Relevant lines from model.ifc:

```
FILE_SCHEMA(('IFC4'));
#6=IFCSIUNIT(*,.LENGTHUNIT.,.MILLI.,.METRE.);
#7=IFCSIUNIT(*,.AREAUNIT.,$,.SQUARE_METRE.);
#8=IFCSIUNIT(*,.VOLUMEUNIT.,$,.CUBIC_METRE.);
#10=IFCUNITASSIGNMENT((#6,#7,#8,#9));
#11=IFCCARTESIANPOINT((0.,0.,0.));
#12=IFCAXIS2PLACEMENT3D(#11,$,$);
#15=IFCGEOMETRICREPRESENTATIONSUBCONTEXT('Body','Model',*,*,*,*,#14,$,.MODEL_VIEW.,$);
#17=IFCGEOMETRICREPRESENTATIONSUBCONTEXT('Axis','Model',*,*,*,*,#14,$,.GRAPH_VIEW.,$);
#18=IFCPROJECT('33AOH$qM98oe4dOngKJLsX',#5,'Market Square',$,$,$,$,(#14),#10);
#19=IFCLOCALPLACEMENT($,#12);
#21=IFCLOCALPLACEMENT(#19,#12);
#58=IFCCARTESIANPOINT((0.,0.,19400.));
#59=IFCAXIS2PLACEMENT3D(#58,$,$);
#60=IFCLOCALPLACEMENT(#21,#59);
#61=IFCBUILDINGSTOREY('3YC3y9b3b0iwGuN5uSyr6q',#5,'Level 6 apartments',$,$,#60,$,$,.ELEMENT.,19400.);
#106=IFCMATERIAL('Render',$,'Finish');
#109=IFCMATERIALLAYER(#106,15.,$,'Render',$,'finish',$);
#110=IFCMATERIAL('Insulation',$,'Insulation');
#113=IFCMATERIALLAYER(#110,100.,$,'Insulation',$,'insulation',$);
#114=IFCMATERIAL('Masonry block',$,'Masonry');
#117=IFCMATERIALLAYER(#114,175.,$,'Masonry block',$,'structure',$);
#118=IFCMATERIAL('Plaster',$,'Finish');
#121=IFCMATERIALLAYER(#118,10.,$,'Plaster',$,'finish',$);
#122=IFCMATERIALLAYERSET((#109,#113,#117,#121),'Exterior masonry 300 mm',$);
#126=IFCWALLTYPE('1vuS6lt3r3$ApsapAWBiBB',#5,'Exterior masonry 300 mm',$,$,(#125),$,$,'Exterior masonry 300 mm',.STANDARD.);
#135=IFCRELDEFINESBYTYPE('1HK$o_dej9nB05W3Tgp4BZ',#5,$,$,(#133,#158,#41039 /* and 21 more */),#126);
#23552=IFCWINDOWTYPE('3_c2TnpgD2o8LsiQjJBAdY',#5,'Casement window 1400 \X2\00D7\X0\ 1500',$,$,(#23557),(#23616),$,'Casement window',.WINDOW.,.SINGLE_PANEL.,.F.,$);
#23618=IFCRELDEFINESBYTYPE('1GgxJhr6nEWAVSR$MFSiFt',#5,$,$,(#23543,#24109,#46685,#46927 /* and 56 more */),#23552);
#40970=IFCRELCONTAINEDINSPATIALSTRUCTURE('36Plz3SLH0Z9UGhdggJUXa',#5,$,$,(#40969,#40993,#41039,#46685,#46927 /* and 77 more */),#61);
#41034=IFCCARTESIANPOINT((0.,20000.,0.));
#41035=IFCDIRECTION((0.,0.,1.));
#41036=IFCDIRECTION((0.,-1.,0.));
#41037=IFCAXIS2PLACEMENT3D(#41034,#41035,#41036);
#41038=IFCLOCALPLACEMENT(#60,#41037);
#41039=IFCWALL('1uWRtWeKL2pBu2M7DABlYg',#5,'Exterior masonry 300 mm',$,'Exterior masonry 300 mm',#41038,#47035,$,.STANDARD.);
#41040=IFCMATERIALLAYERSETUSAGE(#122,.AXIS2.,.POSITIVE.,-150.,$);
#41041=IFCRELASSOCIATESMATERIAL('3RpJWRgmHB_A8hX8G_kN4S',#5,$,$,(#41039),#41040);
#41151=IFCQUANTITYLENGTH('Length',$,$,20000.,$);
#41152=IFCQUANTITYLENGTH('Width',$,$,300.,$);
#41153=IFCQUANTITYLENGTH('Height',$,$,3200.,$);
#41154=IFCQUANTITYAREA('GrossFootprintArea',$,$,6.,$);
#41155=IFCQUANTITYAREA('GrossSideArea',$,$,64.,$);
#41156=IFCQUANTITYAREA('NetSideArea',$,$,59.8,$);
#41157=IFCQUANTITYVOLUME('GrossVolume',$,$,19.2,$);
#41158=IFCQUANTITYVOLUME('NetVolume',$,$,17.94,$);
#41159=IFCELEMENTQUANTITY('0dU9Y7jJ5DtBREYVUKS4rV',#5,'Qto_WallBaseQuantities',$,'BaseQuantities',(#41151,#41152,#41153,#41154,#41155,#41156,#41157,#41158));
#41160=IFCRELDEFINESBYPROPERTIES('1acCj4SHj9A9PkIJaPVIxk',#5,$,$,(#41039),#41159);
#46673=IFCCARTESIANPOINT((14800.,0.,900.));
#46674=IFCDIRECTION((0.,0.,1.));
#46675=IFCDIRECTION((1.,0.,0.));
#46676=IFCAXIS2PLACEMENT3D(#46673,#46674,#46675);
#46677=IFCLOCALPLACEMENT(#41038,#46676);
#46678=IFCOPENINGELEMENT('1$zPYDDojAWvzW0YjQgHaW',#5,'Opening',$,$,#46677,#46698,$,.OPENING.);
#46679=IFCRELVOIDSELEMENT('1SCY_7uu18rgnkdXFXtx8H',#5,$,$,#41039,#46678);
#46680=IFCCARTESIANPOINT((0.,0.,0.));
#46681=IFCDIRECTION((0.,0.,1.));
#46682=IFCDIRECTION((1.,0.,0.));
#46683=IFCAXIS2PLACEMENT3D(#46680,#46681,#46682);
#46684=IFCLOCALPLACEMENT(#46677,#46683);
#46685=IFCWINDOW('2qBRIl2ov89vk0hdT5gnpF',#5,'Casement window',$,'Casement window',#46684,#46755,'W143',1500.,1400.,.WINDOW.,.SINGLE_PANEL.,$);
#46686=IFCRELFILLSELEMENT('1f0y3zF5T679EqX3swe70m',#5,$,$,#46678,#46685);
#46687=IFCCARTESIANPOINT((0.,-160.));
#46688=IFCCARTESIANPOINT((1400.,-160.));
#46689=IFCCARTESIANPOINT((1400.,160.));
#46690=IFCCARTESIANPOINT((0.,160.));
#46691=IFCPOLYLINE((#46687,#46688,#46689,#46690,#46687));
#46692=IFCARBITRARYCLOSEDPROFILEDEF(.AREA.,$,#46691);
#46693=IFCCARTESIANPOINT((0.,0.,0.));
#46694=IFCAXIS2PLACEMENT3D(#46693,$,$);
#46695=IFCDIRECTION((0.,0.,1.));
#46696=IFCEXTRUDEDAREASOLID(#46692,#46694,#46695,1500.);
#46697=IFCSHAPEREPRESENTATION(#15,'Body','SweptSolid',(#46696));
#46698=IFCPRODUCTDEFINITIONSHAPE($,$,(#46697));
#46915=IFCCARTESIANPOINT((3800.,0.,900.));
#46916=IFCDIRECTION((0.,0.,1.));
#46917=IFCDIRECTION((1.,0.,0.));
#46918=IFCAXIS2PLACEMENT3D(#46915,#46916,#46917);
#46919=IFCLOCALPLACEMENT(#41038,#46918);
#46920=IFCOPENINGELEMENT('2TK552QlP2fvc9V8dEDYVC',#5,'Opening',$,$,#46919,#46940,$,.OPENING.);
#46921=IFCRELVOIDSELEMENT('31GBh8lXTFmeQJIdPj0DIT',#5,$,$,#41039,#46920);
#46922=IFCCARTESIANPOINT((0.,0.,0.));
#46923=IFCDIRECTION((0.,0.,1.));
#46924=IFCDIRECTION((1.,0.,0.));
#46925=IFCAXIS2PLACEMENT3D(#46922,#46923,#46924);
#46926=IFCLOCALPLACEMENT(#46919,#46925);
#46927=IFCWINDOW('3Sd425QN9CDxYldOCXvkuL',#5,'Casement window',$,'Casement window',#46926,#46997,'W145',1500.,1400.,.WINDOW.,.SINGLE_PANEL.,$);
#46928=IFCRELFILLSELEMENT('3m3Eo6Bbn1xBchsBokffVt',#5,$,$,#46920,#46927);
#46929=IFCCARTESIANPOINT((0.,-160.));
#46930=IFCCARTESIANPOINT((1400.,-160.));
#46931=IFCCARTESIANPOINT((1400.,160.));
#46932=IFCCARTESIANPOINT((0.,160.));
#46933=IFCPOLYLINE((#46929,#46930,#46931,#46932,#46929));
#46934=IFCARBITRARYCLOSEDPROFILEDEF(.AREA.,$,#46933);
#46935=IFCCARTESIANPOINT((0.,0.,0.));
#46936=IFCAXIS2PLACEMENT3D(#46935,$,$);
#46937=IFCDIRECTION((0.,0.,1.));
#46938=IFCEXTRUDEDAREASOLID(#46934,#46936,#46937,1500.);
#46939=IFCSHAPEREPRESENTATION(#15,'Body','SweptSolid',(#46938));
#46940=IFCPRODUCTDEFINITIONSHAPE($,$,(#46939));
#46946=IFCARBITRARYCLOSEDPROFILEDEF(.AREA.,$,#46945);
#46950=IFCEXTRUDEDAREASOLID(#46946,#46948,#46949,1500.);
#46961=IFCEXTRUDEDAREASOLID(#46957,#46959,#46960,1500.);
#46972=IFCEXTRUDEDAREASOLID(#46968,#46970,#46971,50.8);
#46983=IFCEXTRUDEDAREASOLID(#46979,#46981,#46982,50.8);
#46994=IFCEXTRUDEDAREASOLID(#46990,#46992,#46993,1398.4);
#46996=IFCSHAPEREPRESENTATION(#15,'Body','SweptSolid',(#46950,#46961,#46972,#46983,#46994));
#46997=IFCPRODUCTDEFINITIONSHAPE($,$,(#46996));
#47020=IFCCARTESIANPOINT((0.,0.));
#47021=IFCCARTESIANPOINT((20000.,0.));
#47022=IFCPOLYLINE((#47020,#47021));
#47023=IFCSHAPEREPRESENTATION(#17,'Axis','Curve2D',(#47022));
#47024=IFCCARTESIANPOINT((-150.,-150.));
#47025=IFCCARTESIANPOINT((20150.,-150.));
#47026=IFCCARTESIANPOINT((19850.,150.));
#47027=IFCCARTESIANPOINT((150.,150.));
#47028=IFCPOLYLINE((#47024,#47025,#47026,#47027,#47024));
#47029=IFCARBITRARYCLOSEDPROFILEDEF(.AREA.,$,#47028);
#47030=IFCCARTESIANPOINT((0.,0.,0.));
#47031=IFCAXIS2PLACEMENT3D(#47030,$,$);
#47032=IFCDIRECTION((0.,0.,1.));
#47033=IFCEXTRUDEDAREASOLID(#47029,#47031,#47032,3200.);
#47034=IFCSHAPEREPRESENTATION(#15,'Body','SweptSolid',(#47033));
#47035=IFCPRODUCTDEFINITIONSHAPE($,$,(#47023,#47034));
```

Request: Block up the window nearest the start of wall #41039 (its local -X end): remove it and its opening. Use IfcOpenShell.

```python
import ifcopenshell
import ifcopenshell.api.feature
import ifcopenshell.api.pset
import ifcopenshell.api.root
import ifcopenshell.geom
import ifcopenshell.util.element
import ifcopenshell.util.shape
import ifcopenshell.util.unit

model = ifcopenshell.open("model.ifc")
area_scale = ifcopenshell.util.unit.calculate_unit_scale(model, "AREAUNIT")
volume_scale = ifcopenshell.util.unit.calculate_unit_scale(model, "VOLUMEUNIT")
settings = ifcopenshell.geom.settings()


def volume(element):
    """Net volume in cubic metres, openings subtracted."""
    shape = ifcopenshell.geom.create_shape(settings, element)
    return ifcopenshell.util.shape.get_volume(shape.geometry)


window = model.by_guid("3Sd425QN9CDxYldOCXvkuL")
opening = window.FillsVoids[0].RelatingOpeningElement
wall = opening.VoidsElements[0].RelatingBuildingElement
before = volume(wall)

ifcopenshell.api.root.remove_product(model, product=window)
ifcopenshell.api.feature.remove_feature(model, feature=opening)

after = volume(wall)
thickness = 0.3  # wall thickness in metres

# Update the wall's stored quantities.
qto = model.by_id(ifcopenshell.util.element.get_pset(wall, "Qto_WallBaseQuantities", should_inherit=False)["id"])
ifcopenshell.api.pset.edit_qto(model, qto=qto, properties={
    "NetSideArea": after / thickness / area_scale,
    "NetVolume": after / volume_scale,
})

print(f"wall volume {before:.3f} -> {after:.3f} m3")

model.write("model_rev.ifc")
```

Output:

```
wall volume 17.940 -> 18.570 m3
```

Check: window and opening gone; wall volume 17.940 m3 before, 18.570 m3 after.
